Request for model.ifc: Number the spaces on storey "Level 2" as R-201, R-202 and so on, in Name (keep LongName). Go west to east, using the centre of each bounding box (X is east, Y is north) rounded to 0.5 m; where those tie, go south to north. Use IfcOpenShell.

First a look at what the model holds.

```python
import ifcopenshell
import ifcopenshell.util.element
import ifcopenshell.util.placement

model = ifcopenshell.open("model.ifc")
print(model.schema)
storey = next(s for s in model.by_type("IfcBuildingStorey") if s.Name == "Level 2")
spaces = [e for e in ifcopenshell.util.element.get_decomposition(storey) if e.is_a("IfcSpace")]
for e in sorted(spaces, key=lambda e: e.id()):
    origin = ifcopenshell.util.placement.get_local_placement(e.ObjectPlacement)[:3, 3]
    print(e.id(), e.Name, e.LongName, origin.round(2) + 0.0, sep=" | ")
```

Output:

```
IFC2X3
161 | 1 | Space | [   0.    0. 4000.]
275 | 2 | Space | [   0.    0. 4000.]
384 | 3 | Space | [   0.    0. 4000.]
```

```python
import ifcopenshell
import ifcopenshell.geom
import ifcopenshell.util.element
import ifcopenshell.util.shape

model = ifcopenshell.open("model.ifc")
settings = ifcopenshell.geom.settings()
settings.set("use-world-coords", True)


def centre(element):
    shape = ifcopenshell.geom.create_shape(settings, element)
    return ifcopenshell.util.shape.get_bbox_centroid(shape.geometry)


storey = next(s for s in model.by_type("IfcBuildingStorey") if s.Name == "Level 2")
spaces = [e for e in ifcopenshell.util.element.get_decomposition(storey) if e.is_a("IfcSpace")]

# Insertion points can sit at a corner or the storey origin, so sort by the geometry (in metres).
centres = {e: centre(e) for e in spaces}
spaces.sort(key=lambda e: (round(centres[e][0] / 0.5), centres[e][1]))

for i, e in enumerate(spaces, start=1):
    number = f"R-2{i:02d}"
    e.Name = number
    print(e.id(), number)

model.write("model_rev.ifc")
```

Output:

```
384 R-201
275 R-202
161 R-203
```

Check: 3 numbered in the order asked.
